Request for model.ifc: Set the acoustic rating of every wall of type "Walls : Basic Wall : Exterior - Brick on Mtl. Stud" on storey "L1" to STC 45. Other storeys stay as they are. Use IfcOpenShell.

First a look at what the model holds.

```python
import ifcopenshell
import ifcopenshell.util.element

model = ifcopenshell.open("model.ifc")
print(model.schema)
storey = next(s for s in model.by_type("IfcBuildingStorey") if s.Name == "L1")
walls = [e for e in ifcopenshell.util.element.get_decomposition(storey) if e.is_a("IfcWall")]
seen = {}
for e in walls:
    element_type = ifcopenshell.util.element.get_type(e)
    key = (element_type.Name if element_type != e and element_type else None, ifcopenshell.util.element.get_pset(e, "Pset_WallCommon", "AcousticRating"))
    seen[key] = seen.get(key, 0) + 1
for (name, value), count in sorted(seen.items(), key=str):
    print(count, "x", name, "|", value)
```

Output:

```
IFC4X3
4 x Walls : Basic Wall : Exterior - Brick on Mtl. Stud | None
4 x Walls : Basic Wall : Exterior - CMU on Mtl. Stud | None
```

```python
import ifcopenshell
import ifcopenshell.api.pset
import ifcopenshell.util.element

model = ifcopenshell.open("model.ifc")

storey = next(s for s in model.by_type("IfcBuildingStorey") if s.Name == "L1")
walls = [e for e in ifcopenshell.util.element.get_decomposition(storey) if e.is_a("IfcWall")]

count = 0
for e in walls:
    element_type = ifcopenshell.util.element.get_type(e)
    if element_type in (None, e) or element_type.Name != "Walls : Basic Wall : Exterior - Brick on Mtl. Stud":
        continue
    # add_pset returns the element's existing set when there is one.
    pset = ifcopenshell.api.pset.add_pset(model, product=e, name="Pset_WallCommon")
    ifcopenshell.api.pset.edit_pset(model, pset=pset, properties={"AcousticRating": "STC 45"})
    count += 1

print(count, "walls updated")

model.write("model_v2.ifc")
```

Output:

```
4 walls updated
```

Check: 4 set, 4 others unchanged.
